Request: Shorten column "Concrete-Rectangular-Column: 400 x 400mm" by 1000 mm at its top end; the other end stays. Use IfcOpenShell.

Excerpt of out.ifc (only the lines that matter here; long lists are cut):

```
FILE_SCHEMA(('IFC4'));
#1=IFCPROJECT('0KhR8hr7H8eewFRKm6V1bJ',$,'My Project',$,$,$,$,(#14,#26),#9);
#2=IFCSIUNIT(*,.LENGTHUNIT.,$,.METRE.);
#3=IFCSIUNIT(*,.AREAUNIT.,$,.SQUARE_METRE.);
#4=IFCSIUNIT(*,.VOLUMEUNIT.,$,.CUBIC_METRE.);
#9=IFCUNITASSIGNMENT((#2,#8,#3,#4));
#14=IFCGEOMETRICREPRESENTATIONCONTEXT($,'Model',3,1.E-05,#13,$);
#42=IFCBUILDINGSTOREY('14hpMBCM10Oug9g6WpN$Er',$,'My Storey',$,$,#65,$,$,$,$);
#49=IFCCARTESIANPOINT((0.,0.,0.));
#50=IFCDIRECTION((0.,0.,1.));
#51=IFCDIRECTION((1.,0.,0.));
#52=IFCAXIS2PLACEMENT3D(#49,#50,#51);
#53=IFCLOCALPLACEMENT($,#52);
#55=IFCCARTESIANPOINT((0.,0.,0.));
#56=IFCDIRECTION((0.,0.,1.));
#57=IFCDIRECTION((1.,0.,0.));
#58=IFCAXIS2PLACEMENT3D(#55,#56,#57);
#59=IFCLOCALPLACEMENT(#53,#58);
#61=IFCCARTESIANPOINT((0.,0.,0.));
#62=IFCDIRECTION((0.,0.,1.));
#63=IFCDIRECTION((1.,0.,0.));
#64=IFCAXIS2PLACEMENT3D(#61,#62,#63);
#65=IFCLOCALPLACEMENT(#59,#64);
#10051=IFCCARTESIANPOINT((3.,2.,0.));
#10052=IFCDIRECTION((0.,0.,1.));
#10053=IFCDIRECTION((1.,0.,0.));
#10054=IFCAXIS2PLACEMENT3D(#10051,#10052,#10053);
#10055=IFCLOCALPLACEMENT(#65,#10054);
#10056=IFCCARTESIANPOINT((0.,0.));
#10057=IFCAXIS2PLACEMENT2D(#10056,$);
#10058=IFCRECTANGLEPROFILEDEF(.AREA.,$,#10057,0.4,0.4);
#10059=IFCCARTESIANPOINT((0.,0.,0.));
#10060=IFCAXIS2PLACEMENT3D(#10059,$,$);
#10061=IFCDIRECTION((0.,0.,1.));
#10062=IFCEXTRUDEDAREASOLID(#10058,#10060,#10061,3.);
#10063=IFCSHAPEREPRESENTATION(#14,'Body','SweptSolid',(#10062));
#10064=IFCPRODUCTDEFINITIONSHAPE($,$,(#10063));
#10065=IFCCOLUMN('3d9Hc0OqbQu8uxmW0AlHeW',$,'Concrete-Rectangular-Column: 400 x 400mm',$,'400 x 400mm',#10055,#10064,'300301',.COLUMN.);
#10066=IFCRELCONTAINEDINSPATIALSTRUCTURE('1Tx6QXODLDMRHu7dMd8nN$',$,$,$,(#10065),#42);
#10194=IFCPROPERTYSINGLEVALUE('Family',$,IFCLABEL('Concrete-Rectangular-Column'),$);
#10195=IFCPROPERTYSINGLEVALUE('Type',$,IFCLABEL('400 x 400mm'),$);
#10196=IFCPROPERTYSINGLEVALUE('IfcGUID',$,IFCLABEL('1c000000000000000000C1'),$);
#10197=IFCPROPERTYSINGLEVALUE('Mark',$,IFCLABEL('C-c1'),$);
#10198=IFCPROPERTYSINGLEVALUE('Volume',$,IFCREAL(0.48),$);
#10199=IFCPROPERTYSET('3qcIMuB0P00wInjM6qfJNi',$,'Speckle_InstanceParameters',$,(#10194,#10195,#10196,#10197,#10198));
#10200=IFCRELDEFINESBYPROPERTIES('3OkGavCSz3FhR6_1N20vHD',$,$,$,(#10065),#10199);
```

```python
import ifcopenshell
import ifcopenshell.api.pset
import ifcopenshell.util.element

model = ifcopenshell.open("out.ifc")

member = model.by_id(10065)
change = -1.0

# The extrusion runs towards the end named, so only its depth changes.
body = next(r for r in member.Representation.Representations if r.RepresentationIdentifier == "Body")
solid = body.Items[0]
old_length = solid.Depth
solid.Depth += change

# Update the stored length and volume.
pset = model.by_id(ifcopenshell.util.element.get_pset(member, "Speckle_InstanceParameters", should_inherit=False)["id"])
ifcopenshell.api.pset.edit_pset(model, pset=pset, properties={
    "Volume": model.create_entity("IfcReal", ifcopenshell.util.element.get_pset(member, "Speckle_InstanceParameters", "Volume") * solid.Depth / old_length),
})

print(f"length {old_length:g} -> {solid.Depth:g}")

model.write("out_rev.ifc")
```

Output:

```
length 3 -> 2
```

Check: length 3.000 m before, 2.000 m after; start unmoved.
